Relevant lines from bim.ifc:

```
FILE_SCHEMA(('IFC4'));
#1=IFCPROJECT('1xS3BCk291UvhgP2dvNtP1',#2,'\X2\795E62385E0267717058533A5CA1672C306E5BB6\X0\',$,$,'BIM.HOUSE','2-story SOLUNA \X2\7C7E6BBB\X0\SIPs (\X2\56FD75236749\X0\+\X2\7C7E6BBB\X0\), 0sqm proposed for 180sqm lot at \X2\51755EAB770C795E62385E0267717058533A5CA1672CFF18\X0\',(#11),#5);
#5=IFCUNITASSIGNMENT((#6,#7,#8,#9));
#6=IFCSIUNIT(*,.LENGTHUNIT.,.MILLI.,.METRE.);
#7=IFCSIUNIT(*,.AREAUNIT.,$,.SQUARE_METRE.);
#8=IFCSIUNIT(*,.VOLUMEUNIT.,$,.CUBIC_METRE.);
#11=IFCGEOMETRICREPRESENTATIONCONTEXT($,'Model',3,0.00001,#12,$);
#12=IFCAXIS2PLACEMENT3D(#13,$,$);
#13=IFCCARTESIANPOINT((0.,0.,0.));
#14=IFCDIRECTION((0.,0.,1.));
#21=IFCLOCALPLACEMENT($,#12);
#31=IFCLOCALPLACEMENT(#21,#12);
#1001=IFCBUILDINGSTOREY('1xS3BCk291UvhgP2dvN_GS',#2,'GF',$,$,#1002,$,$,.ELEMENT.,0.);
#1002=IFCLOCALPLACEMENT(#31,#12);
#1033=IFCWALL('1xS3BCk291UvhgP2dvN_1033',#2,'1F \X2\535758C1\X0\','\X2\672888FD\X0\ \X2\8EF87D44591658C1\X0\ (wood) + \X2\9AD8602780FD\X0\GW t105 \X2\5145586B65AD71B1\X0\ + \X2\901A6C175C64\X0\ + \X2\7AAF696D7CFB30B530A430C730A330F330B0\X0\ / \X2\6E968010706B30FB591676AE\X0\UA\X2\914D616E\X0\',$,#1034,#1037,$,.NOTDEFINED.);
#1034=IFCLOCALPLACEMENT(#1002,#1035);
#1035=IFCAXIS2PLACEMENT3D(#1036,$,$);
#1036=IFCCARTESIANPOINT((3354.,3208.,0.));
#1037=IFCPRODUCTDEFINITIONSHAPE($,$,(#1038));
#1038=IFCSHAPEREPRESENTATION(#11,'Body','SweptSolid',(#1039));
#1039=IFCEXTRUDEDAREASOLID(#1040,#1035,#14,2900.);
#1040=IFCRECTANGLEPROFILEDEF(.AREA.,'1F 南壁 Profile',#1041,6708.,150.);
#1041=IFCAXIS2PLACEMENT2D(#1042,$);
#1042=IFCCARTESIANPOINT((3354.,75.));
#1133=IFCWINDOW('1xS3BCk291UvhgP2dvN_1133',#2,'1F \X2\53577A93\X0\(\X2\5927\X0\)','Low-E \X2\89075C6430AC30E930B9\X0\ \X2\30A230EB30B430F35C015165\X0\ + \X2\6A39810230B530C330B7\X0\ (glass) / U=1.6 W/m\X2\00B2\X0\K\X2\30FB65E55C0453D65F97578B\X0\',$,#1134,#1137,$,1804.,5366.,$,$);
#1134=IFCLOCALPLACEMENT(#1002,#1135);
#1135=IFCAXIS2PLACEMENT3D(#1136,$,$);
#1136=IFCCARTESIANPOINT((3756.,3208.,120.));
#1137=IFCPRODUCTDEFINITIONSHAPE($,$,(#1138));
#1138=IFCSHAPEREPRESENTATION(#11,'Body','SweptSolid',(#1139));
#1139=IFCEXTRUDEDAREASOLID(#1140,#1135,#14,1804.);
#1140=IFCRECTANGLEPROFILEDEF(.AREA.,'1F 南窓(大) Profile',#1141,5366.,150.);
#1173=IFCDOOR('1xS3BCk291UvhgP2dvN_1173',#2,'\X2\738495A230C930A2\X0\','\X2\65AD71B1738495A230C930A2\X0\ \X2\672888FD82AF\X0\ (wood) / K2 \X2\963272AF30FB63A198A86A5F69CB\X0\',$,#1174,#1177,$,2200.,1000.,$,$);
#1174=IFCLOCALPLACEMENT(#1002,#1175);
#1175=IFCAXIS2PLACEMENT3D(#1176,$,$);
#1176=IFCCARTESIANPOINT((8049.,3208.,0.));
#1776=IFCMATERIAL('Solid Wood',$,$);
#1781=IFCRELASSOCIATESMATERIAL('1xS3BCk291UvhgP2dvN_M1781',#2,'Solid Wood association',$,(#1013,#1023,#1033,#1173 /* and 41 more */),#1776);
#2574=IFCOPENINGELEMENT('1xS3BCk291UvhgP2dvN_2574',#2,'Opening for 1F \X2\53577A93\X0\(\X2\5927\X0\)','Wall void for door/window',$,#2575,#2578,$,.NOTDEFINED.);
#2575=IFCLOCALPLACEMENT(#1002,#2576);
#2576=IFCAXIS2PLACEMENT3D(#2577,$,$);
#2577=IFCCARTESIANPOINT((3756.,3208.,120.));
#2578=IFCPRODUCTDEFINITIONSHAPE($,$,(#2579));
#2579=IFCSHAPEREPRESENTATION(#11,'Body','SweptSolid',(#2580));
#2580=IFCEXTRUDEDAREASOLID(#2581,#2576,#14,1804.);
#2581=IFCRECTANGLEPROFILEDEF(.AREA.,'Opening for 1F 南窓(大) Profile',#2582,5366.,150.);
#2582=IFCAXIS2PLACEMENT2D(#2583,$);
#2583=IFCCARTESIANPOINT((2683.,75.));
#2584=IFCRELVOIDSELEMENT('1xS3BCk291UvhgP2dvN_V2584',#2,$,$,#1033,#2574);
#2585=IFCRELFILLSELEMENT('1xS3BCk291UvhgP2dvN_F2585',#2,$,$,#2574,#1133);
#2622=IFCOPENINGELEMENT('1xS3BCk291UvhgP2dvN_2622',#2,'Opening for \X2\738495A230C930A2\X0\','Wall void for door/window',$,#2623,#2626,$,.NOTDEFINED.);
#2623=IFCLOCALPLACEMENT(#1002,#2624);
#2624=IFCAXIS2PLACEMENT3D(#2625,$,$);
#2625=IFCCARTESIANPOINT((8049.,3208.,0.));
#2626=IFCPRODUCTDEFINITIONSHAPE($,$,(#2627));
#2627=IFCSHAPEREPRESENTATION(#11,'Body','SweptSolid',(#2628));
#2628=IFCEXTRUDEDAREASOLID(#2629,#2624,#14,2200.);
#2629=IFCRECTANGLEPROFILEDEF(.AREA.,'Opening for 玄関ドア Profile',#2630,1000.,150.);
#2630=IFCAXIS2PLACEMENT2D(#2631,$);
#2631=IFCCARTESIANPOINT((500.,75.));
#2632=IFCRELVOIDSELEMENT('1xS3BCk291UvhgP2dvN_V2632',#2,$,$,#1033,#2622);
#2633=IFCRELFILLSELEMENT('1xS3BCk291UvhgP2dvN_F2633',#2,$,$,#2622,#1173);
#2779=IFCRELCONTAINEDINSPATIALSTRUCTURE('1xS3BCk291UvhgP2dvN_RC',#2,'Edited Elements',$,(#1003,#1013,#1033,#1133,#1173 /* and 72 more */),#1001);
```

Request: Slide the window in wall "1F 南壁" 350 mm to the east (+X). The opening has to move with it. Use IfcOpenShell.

```python
import ifcopenshell
import ifcopenshell.api.geometry
import ifcopenshell.util.placement
import ifcopenshell.util.unit

model = ifcopenshell.open("bim.ifc")
unit_scale = ifcopenshell.util.unit.calculate_unit_scale(model)

window = model.by_id(1133)
opening = window.FillsVoids[0].RelatingOpeningElement
wall = opening.VoidsElements[0].RelatingBuildingElement

wall_matrix = ifcopenshell.util.placement.get_local_placement(wall.ObjectPlacement)
shift = wall_matrix[:3, 0] * 0.35 / unit_scale
before = ifcopenshell.util.placement.get_local_placement(window.ObjectPlacement)[:3, 3].copy()

# The window is not placed relative to its opening, so move both.
for product in (opening, window):
    matrix = ifcopenshell.util.placement.get_local_placement(product.ObjectPlacement)
    matrix[:3, 3] += shift
    ifcopenshell.api.geometry.edit_object_placement(model, product=product, matrix=matrix, is_si=False)

after = ifcopenshell.util.placement.get_local_placement(window.ObjectPlacement)[:3, 3]
print("window moved by", (after - before).round(3) + 0.0)

model.write("bim-out.ifc")
```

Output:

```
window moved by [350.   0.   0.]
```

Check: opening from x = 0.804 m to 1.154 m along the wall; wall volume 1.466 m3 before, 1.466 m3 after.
